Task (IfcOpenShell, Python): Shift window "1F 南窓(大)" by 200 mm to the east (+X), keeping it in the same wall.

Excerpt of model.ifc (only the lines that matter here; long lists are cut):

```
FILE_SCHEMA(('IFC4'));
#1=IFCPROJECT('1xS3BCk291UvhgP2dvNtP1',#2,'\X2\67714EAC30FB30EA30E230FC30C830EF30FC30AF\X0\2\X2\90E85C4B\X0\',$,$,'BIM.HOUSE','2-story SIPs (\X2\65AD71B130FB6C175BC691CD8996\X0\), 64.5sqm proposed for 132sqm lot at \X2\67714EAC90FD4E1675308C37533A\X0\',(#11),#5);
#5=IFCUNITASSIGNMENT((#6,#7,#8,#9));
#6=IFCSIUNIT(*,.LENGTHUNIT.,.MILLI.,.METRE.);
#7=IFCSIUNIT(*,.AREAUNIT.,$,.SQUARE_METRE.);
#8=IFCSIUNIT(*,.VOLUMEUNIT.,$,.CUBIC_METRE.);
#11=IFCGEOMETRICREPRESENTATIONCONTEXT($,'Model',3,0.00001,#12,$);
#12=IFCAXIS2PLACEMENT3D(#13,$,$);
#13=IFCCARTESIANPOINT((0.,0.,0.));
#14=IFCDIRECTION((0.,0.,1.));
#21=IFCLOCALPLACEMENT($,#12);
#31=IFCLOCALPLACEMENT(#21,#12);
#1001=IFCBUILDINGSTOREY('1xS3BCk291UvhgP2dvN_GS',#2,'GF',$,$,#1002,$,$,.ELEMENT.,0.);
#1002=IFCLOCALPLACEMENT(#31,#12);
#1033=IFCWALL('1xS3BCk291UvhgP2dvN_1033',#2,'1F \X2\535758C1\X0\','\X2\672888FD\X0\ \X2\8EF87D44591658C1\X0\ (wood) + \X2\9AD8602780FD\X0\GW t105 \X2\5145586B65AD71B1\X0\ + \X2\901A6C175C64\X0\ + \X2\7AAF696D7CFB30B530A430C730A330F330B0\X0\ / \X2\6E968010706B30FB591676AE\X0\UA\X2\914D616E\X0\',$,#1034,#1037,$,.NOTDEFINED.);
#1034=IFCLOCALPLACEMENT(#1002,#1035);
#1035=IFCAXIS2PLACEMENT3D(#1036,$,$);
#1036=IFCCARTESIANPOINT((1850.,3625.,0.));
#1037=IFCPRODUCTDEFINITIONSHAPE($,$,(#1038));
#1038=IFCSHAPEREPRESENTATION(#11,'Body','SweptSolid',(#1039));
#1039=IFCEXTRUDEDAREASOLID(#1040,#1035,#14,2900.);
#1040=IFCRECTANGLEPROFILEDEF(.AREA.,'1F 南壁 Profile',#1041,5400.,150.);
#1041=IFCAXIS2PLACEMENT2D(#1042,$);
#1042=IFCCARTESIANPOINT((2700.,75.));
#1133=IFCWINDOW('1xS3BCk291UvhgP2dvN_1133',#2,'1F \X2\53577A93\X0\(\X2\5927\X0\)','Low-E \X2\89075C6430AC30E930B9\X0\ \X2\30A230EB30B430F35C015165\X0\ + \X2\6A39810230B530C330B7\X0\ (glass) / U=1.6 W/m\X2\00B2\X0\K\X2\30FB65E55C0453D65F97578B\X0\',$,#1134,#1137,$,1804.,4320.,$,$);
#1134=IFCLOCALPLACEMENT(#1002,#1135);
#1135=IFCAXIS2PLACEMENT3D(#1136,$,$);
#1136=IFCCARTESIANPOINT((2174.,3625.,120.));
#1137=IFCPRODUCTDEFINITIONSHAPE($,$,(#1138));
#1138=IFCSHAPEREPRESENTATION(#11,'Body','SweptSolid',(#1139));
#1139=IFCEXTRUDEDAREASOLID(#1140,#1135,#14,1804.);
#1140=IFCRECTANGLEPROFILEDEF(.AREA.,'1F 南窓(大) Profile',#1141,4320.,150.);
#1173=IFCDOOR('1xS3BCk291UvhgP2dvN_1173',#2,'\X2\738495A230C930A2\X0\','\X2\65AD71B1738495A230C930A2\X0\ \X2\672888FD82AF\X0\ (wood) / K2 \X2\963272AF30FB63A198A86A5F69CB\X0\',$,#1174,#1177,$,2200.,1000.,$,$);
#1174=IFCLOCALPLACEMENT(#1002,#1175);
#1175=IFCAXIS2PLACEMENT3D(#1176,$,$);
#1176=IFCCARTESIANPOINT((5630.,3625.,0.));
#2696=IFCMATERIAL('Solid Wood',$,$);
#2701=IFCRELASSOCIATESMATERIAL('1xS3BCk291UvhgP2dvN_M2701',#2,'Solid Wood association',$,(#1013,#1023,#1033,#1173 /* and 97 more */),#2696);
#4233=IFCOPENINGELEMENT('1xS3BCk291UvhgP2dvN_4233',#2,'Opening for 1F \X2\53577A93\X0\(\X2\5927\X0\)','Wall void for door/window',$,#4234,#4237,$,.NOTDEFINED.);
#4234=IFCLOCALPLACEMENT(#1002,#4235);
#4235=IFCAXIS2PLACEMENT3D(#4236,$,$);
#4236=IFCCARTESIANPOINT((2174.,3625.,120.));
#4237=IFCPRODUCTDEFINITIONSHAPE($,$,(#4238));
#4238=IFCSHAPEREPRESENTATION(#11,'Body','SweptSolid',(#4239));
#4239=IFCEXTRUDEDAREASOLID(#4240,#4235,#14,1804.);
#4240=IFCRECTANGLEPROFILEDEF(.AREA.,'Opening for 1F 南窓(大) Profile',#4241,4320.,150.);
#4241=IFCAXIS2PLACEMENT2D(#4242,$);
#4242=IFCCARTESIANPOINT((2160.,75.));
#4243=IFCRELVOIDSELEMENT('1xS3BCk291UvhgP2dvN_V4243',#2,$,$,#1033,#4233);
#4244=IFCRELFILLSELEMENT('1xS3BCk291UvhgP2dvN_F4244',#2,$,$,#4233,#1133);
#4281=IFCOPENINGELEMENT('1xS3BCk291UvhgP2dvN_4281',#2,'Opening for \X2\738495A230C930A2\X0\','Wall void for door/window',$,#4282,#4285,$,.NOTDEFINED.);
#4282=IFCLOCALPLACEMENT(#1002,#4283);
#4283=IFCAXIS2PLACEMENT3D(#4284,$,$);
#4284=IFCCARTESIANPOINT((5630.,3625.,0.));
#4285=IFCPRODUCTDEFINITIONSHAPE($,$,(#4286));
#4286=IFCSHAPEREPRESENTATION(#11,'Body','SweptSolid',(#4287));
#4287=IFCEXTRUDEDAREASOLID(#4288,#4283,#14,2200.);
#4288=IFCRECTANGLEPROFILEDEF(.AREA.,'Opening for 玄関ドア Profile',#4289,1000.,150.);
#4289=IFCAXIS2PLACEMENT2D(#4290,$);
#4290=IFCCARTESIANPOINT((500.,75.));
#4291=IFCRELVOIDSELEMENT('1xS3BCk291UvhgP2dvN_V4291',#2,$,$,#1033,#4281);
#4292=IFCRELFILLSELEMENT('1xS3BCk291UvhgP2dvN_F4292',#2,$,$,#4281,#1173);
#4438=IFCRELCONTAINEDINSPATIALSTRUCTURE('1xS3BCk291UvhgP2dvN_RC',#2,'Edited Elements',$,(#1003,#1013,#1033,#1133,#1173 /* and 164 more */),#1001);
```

```python
import ifcopenshell
import ifcopenshell.api.geometry
import ifcopenshell.util.placement

model = ifcopenshell.open("model.ifc")

window = model.by_guid("1xS3BCk291UvhgP2dvN_1133")
opening = window.FillsVoids[0].RelatingOpeningElement
wall = opening.VoidsElements[0].RelatingBuildingElement

wall_matrix = ifcopenshell.util.placement.get_local_placement(wall.ObjectPlacement)
shift = wall_matrix[:3, 0] * 200.0
before = ifcopenshell.util.placement.get_local_placement(window.ObjectPlacement)[:3, 3].copy()

# The window is not placed relative to its opening, so move both.
for product in (opening, window):
    matrix = ifcopenshell.util.placement.get_local_placement(product.ObjectPlacement)
    matrix[:3, 3] += shift
    ifcopenshell.api.geometry.edit_object_placement(model, product=product, matrix=matrix, is_si=False)

after = ifcopenshell.util.placement.get_local_placement(window.ObjectPlacement)[:3, 3]
print("window moved by", (after - before).round(3) + 0.0)

model.write("model_rev.ifc")
```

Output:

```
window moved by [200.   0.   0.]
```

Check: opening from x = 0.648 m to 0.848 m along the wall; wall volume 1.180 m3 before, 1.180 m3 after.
